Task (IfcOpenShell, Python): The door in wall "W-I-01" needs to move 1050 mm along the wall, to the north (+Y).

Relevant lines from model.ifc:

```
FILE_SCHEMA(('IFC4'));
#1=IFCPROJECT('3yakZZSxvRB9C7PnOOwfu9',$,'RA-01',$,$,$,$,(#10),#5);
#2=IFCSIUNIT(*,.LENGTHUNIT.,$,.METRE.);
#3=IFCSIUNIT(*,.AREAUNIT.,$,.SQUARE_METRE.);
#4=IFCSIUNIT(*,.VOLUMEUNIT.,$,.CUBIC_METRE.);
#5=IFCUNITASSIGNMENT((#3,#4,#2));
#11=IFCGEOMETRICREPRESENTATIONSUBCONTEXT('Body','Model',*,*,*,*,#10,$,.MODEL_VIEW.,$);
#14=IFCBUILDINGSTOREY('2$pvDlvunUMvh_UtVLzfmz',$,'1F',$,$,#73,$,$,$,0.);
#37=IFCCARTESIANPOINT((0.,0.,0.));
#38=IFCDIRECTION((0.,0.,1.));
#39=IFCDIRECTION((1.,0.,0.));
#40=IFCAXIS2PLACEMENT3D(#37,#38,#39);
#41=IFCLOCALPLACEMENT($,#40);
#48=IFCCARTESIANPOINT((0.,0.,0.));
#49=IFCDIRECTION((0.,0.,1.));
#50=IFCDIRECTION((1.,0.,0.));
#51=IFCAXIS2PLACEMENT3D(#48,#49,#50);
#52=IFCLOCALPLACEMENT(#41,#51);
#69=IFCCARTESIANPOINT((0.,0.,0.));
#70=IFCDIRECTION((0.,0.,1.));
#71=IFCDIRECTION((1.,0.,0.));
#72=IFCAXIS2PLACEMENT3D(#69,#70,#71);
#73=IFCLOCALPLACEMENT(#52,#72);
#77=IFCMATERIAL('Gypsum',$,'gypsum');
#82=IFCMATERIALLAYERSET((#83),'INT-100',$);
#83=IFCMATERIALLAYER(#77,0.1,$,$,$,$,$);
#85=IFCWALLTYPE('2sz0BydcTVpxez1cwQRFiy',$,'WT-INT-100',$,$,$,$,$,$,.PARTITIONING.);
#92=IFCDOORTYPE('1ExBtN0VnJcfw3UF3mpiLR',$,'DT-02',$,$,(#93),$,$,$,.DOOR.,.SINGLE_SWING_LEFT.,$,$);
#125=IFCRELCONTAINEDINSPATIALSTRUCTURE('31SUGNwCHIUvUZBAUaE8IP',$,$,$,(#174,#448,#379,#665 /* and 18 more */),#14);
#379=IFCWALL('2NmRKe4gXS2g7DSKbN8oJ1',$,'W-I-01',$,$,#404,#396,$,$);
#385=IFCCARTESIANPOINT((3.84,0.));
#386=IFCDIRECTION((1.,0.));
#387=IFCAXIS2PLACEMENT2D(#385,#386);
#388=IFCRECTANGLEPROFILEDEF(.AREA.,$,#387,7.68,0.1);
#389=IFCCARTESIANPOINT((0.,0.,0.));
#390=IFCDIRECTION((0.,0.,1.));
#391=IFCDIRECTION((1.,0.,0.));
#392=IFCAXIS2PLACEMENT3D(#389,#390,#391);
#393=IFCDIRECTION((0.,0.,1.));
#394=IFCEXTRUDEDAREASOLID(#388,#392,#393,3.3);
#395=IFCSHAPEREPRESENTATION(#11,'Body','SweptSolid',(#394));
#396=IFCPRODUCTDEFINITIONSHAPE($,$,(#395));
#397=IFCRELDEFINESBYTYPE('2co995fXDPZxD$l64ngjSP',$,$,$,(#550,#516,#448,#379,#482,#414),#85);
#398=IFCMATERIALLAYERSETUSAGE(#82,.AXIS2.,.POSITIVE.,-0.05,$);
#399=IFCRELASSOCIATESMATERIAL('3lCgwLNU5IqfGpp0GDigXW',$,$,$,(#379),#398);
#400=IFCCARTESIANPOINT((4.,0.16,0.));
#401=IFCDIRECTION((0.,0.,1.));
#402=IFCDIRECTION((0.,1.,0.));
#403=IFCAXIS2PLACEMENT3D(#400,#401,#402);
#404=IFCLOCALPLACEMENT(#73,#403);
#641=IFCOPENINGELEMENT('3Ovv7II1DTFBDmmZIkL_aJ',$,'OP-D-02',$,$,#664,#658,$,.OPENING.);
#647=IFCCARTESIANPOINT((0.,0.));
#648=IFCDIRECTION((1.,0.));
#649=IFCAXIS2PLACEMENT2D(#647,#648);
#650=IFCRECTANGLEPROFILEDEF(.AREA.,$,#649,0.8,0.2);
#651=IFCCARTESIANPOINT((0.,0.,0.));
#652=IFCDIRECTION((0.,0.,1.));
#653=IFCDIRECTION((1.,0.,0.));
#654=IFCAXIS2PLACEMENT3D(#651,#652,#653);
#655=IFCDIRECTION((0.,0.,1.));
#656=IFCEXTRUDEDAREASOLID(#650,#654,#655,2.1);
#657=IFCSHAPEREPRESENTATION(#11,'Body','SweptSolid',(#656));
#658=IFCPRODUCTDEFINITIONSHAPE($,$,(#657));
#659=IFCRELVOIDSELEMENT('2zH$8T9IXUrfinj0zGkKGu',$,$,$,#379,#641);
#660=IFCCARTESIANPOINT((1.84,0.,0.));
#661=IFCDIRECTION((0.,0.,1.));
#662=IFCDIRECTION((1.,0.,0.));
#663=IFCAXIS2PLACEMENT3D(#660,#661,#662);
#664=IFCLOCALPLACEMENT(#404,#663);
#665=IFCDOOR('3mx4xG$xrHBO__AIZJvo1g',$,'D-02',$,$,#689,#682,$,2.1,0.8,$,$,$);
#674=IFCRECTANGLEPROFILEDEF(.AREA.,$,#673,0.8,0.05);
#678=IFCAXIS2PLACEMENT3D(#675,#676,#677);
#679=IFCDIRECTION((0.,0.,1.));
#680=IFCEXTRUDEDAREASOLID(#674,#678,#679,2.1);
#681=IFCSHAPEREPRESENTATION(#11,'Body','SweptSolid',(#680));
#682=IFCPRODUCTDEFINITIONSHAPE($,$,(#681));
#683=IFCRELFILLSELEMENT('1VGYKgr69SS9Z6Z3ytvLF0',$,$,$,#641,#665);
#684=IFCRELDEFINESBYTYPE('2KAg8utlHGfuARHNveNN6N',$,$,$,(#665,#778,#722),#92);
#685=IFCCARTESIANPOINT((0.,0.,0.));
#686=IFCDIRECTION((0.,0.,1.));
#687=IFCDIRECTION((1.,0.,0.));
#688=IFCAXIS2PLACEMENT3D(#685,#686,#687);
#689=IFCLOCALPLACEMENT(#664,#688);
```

```python
import ifcopenshell
import ifcopenshell.api.geometry
import ifcopenshell.util.placement

model = ifcopenshell.open("model.ifc")

door = model.by_guid("3mx4xG$xrHBO__AIZJvo1g")
opening = door.FillsVoids[0].RelatingOpeningElement
wall = opening.VoidsElements[0].RelatingBuildingElement

wall_matrix = ifcopenshell.util.placement.get_local_placement(wall.ObjectPlacement)
shift = wall_matrix[:3, 0] * 1.05
before = ifcopenshell.util.placement.get_local_placement(door.ObjectPlacement)[:3, 3].copy()

# The door is placed relative to its opening, so it follows when the opening moves.
matrix = ifcopenshell.util.placement.get_local_placement(opening.ObjectPlacement)
matrix[:3, 3] += shift
ifcopenshell.api.geometry.edit_object_placement(
    model, product=opening, matrix=matrix, is_si=False, should_transform_children=True
)

after = ifcopenshell.util.placement.get_local_placement(door.ObjectPlacement)[:3, 3]
print("door moved by", (after - before).round(3) + 0.0)

model.write("model_v2.ifc")
```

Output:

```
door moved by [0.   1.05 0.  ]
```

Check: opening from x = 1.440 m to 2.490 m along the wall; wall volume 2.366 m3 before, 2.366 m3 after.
